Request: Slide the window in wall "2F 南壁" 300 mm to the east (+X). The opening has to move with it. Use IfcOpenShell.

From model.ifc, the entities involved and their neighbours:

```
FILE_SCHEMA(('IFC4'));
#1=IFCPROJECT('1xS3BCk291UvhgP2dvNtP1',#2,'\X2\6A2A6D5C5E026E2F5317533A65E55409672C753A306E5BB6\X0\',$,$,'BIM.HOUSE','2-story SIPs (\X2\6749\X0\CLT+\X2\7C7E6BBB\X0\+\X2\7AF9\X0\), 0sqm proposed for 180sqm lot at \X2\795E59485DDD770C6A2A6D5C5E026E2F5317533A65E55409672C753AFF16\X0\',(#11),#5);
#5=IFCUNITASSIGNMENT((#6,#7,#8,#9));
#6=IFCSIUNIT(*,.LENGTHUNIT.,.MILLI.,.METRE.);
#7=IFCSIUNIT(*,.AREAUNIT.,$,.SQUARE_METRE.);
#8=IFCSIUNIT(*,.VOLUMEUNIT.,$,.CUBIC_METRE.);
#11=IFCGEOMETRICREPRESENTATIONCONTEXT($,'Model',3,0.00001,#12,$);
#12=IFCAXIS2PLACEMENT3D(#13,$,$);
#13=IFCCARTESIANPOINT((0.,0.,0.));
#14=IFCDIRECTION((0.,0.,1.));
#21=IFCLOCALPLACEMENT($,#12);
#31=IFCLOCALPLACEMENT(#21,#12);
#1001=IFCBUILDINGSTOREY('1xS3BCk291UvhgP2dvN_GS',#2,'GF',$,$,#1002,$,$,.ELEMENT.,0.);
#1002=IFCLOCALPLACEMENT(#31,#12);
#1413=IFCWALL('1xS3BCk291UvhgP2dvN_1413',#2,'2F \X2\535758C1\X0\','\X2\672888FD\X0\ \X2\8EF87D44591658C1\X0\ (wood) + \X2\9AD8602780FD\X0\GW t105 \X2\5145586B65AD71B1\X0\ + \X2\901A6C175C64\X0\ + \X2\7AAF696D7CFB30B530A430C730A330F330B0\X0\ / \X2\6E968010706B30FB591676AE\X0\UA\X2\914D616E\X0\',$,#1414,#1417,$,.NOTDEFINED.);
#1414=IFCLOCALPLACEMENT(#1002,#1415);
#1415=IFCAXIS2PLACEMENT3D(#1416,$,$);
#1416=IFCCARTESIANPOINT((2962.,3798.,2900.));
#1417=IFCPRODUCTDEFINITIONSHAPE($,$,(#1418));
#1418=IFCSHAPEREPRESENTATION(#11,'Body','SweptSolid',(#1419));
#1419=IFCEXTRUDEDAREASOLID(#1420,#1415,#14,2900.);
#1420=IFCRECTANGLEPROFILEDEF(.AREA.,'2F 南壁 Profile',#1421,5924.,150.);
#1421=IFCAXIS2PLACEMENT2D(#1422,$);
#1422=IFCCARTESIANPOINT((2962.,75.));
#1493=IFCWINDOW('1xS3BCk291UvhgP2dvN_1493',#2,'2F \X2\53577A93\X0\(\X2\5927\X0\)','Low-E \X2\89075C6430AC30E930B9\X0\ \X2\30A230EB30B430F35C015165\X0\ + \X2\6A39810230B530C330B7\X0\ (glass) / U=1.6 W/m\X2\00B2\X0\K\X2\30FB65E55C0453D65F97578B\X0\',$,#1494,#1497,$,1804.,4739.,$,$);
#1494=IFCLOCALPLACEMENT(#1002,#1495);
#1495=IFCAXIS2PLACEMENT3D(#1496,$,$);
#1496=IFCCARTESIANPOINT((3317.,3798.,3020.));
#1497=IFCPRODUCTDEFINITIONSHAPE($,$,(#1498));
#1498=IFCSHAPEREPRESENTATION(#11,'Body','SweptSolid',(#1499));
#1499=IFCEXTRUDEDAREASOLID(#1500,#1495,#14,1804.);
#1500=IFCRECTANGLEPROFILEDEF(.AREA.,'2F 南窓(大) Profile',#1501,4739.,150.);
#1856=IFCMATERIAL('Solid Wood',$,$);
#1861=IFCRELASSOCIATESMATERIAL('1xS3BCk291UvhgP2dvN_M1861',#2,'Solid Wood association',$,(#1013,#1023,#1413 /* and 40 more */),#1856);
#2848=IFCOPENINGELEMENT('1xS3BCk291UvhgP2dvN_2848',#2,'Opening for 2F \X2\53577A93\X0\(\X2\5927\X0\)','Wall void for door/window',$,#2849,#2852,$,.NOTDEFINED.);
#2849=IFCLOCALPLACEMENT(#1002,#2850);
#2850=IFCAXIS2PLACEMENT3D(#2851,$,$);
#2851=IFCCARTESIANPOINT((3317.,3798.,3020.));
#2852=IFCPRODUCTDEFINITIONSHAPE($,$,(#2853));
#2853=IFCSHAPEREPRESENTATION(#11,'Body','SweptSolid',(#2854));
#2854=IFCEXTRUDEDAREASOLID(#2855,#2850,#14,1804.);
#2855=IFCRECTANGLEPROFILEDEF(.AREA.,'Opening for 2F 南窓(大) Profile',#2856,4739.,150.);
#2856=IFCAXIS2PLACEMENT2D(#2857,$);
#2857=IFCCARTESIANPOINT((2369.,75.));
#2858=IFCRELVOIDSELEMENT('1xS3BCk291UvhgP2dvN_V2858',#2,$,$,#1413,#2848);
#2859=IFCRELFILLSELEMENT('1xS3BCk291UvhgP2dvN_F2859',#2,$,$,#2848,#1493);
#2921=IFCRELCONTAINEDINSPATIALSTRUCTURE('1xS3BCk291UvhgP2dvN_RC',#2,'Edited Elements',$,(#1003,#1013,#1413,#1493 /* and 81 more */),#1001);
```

```python
import ifcopenshell
import ifcopenshell.api.geometry
import ifcopenshell.util.placement
import ifcopenshell.util.unit

model = ifcopenshell.open("model.ifc")
unit_scale = ifcopenshell.util.unit.calculate_unit_scale(model)

window = model.by_id(1493)
opening = window.FillsVoids[0].RelatingOpeningElement
wall = opening.VoidsElements[0].RelatingBuildingElement

wall_matrix = ifcopenshell.util.placement.get_local_placement(wall.ObjectPlacement)
shift = wall_matrix[:3, 0] * 0.3 / unit_scale
before = ifcopenshell.util.placement.get_local_placement(window.ObjectPlacement)[:3, 3].copy()

# The window is not placed relative to its opening, so move both.
for product in (opening, window):
    matrix = ifcopenshell.util.placement.get_local_placement(product.ObjectPlacement)
    matrix[:3, 3] += shift
    ifcopenshell.api.geometry.edit_object_placement(model, product=product, matrix=matrix, is_si=False)

after = ifcopenshell.util.placement.get_local_placement(window.ObjectPlacement)[:3, 3]
print("window moved by", (after - before).round(3) + 0.0)

model.write("model_rev.ifc")
```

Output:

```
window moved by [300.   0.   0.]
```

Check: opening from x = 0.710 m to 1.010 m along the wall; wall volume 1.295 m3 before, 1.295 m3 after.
